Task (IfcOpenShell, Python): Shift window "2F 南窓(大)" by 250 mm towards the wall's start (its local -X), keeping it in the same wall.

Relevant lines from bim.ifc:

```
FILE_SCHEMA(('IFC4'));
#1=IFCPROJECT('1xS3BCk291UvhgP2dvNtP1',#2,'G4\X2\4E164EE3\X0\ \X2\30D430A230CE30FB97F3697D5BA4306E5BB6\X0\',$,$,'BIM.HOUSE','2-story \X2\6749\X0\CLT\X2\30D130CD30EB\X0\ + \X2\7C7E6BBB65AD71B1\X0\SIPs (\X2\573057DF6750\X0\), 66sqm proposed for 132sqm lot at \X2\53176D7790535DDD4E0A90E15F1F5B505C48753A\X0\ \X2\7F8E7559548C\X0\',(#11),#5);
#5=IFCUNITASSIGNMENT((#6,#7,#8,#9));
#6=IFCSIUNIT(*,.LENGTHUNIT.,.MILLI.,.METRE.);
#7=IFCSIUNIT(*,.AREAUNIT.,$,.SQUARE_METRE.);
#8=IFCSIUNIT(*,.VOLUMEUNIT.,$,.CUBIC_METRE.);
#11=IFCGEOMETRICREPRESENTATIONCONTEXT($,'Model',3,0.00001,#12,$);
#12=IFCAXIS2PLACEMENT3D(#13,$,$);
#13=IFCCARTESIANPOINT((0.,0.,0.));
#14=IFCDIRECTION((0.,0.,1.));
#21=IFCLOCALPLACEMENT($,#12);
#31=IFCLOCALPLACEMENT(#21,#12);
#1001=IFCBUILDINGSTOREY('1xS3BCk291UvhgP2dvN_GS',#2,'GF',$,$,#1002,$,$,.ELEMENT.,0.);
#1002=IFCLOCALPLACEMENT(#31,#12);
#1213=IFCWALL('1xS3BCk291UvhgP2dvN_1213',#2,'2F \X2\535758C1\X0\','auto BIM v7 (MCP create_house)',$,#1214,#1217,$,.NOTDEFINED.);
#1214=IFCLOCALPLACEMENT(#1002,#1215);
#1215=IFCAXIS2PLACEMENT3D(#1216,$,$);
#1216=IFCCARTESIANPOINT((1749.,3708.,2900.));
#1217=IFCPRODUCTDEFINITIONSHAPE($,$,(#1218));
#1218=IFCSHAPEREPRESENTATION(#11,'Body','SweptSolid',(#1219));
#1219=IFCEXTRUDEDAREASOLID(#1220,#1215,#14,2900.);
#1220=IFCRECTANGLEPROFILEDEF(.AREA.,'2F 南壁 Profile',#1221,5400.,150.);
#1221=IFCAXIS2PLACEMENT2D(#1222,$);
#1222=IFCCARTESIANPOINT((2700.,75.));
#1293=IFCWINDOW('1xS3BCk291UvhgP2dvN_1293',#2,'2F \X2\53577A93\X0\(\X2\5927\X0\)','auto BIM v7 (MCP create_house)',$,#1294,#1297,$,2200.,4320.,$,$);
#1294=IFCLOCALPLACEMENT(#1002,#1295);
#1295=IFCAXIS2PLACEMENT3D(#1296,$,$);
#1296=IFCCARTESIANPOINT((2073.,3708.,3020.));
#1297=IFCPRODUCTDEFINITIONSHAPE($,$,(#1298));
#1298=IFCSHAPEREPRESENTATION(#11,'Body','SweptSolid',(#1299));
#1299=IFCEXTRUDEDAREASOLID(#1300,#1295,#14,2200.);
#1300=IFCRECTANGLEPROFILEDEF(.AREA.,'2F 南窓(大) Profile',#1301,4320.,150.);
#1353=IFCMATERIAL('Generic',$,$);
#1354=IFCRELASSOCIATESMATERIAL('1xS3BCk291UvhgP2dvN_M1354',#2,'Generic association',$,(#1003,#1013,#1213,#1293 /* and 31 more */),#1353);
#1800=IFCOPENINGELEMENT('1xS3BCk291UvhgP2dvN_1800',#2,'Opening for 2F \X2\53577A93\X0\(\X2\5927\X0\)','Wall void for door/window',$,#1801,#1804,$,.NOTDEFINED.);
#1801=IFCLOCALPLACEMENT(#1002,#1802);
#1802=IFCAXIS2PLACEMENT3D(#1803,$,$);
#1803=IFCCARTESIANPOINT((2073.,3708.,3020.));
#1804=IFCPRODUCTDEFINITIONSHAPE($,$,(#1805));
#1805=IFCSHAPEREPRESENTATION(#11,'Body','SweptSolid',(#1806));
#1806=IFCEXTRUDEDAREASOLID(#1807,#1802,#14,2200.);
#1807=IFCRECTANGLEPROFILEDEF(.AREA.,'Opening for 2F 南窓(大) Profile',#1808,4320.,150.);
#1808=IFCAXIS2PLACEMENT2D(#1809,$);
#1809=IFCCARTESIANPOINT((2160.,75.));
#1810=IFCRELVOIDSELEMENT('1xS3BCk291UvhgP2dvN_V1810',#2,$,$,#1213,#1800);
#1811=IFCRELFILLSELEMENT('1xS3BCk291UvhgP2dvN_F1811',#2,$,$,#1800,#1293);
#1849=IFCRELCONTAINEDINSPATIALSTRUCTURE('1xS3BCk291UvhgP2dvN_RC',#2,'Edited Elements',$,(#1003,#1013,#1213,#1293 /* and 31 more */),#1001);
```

```python
import ifcopenshell
import ifcopenshell.api.geometry
import ifcopenshell.util.placement

model = ifcopenshell.open("bim.ifc")

window = model.by_guid("1xS3BCk291UvhgP2dvN_1293")
opening = window.FillsVoids[0].RelatingOpeningElement
wall = opening.VoidsElements[0].RelatingBuildingElement

wall_matrix = ifcopenshell.util.placement.get_local_placement(wall.ObjectPlacement)
shift = wall_matrix[:3, 0] * -250.0
before = ifcopenshell.util.placement.get_local_placement(window.ObjectPlacement)[:3, 3].copy()

# The window is not placed relative to its opening, so move both.
for product in (opening, window):
    matrix = ifcopenshell.util.placement.get_local_placement(product.ObjectPlacement)
    matrix[:3, 3] += shift
    ifcopenshell.api.geometry.edit_object_placement(model, product=product, matrix=matrix, is_si=False)

after = ifcopenshell.util.placement.get_local_placement(window.ObjectPlacement)[:3, 3]
print("window moved by", (after - before).round(3) + 0.0)

model.write("bim-out.ifc")
```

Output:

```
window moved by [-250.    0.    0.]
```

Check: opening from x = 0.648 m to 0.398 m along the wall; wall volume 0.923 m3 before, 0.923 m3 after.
